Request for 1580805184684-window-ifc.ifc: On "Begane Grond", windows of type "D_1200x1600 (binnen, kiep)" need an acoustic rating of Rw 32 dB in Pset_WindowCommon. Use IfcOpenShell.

First a look at what the model holds.

```python
import ifcopenshell
import ifcopenshell.util.element

model = ifcopenshell.open("1580805184684-window-ifc.ifc")
print(model.schema)
storey = next(s for s in model.by_type("IfcBuildingStorey") if s.Name == "Begane Grond")
windows = [e for e in ifcopenshell.util.element.get_decomposition(storey) if e.is_a("IfcWindow")]
seen = {}
for e in windows:
    element_type = ifcopenshell.util.element.get_type(e)
    key = (element_type.Name if element_type != e and element_type else None, ifcopenshell.util.element.get_pset(e, "Pset_WindowCommon", "AcousticRating"))
    seen[key] = seen.get(key, 0) + 1
for (name, value), count in sorted(seen.items(), key=str):
    print(count, "x", name, "|", value)
```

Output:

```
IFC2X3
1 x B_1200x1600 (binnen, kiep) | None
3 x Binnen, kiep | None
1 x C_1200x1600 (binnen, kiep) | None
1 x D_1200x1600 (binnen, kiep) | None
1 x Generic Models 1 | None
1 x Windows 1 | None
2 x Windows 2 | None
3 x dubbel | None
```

```python
import ifcopenshell
import ifcopenshell.api.pset
import ifcopenshell.util.element

model = ifcopenshell.open("1580805184684-window-ifc.ifc")

storey = next(s for s in model.by_type("IfcBuildingStorey") if s.Name == "Begane Grond")
windows = [e for e in ifcopenshell.util.element.get_decomposition(storey) if e.is_a("IfcWindow")]

count = 0
for e in windows:
    element_type = ifcopenshell.util.element.get_type(e)
    if element_type in (None, e) or element_type.Name != "D_1200x1600 (binnen, kiep)":
        continue
    # add_pset returns the element's existing set when there is one.
    pset = ifcopenshell.api.pset.add_pset(model, product=e, name="Pset_WindowCommon")
    ifcopenshell.api.pset.edit_pset(model, pset=pset, properties={"AcousticRating": "Rw 32 dB"})
    count += 1

print(count, "windows updated")

model.write("1580805184684-window-ifc_v2.ifc")
```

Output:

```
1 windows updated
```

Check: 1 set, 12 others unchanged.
